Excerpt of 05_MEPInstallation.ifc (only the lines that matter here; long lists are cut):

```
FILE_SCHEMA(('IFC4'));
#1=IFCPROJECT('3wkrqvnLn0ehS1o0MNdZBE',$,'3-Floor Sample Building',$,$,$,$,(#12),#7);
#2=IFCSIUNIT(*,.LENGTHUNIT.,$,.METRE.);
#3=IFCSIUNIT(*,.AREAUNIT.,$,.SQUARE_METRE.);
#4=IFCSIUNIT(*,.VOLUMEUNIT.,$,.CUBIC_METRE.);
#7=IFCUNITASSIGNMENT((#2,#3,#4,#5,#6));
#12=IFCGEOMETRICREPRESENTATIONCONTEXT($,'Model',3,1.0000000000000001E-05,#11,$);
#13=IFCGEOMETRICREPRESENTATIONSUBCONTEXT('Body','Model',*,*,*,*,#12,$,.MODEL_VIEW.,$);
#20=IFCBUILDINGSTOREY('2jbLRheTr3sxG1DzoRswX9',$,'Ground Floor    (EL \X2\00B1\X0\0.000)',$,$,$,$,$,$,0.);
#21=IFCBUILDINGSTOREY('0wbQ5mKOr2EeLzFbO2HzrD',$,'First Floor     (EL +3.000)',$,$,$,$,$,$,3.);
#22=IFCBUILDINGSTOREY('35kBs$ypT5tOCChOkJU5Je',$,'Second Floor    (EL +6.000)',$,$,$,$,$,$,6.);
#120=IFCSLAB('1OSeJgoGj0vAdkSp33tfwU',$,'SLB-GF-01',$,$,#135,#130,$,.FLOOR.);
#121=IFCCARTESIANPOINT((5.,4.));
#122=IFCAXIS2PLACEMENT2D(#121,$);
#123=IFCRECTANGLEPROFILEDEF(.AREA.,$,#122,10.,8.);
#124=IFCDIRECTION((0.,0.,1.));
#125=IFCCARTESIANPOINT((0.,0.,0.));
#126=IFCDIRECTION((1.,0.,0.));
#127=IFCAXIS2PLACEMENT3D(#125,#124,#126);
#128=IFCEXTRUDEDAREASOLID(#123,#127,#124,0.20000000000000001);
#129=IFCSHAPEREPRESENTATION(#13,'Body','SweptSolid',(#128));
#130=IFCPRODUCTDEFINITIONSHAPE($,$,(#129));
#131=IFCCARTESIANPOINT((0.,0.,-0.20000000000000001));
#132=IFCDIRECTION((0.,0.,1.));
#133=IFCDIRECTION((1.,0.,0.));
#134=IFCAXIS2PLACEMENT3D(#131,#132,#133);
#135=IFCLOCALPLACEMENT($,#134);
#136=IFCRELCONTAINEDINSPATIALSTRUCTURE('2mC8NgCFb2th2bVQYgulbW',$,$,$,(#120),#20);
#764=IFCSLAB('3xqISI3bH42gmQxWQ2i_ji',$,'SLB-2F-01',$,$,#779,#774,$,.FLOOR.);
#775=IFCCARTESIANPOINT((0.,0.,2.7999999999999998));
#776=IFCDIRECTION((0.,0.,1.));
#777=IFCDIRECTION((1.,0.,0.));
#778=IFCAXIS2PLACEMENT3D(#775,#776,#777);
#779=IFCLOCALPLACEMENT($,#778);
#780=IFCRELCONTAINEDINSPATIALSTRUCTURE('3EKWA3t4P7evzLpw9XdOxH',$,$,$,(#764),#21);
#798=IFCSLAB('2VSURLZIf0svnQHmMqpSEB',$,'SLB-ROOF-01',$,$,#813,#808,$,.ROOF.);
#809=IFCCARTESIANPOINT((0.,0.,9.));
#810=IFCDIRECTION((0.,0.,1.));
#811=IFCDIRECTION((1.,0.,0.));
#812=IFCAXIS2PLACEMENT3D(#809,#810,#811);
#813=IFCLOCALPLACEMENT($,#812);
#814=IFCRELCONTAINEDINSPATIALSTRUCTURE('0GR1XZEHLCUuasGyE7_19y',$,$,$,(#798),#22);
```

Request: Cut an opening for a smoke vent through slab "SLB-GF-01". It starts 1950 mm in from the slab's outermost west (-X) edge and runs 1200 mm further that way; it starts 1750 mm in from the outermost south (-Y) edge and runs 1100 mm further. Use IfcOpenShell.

```python
import numpy as np
import ifcopenshell
import ifcopenshell.api.feature
import ifcopenshell.api.geometry
import ifcopenshell.api.root
import ifcopenshell.geom
import ifcopenshell.util.placement
import ifcopenshell.util.representation
import ifcopenshell.util.shape
import ifcopenshell.util.unit

model = ifcopenshell.open("05_MEPInstallation.ifc")
unit_scale = ifcopenshell.util.unit.calculate_unit_scale(model)
settings = ifcopenshell.geom.settings()


def volume(element):
    """Net volume in cubic metres, openings subtracted."""
    shape = ifcopenshell.geom.create_shape(settings, element)
    return ifcopenshell.util.shape.get_volume(shape.geometry)


slab = model.by_guid("1OSeJgoGj0vAdkSp33tfwU")
before = volume(slab)

# Extent in the slab's own axes, in metres. The edges named are its -X and -Y sides.
slab_shape = ifcopenshell.geom.create_shape(settings, slab)
vertices = ifcopenshell.util.shape.get_vertices(slab_shape.geometry)
x_min, y_min, bottom = vertices.min(axis=0)
top = vertices[:, 2].max()

opening = ifcopenshell.api.root.create_entity(model, ifc_class="IfcOpeningElement", name="Smoke vent opening", predefined_type="OPENING")
context = ifcopenshell.util.representation.get_context(model, "Model", "Body", "MODEL_VIEW")
width, depth = 1.2, 1.1
outline = [(0.0, 0.0), (width, 0.0), (width, depth), (0.0, depth), (0.0, 0.0)]
# Overshoot both faces by 50 mm so the cut is clean.
shape = ifcopenshell.api.geometry.add_slab_representation(
    model, context=context, depth=top - bottom + 0.1, polyline=outline
)
ifcopenshell.api.geometry.assign_representation(model, product=opening, representation=shape)

matrix = ifcopenshell.util.placement.get_local_placement(slab.ObjectPlacement)
matrix[:, 3] = matrix @ np.append(np.array([x_min + 1.95, y_min + 1.75, bottom - 0.05]) / unit_scale, 1.0)
ifcopenshell.api.geometry.edit_object_placement(model, product=opening, matrix=matrix, is_si=False)
ifcopenshell.api.feature.add_feature(model, feature=opening, element=slab)

after = volume(slab)

print(f"slab volume {before:.3f} -> {after:.3f} m3")

model.write("05_MEPInstallation-out.ifc")
```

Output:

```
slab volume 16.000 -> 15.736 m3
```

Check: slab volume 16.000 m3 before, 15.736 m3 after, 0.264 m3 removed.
